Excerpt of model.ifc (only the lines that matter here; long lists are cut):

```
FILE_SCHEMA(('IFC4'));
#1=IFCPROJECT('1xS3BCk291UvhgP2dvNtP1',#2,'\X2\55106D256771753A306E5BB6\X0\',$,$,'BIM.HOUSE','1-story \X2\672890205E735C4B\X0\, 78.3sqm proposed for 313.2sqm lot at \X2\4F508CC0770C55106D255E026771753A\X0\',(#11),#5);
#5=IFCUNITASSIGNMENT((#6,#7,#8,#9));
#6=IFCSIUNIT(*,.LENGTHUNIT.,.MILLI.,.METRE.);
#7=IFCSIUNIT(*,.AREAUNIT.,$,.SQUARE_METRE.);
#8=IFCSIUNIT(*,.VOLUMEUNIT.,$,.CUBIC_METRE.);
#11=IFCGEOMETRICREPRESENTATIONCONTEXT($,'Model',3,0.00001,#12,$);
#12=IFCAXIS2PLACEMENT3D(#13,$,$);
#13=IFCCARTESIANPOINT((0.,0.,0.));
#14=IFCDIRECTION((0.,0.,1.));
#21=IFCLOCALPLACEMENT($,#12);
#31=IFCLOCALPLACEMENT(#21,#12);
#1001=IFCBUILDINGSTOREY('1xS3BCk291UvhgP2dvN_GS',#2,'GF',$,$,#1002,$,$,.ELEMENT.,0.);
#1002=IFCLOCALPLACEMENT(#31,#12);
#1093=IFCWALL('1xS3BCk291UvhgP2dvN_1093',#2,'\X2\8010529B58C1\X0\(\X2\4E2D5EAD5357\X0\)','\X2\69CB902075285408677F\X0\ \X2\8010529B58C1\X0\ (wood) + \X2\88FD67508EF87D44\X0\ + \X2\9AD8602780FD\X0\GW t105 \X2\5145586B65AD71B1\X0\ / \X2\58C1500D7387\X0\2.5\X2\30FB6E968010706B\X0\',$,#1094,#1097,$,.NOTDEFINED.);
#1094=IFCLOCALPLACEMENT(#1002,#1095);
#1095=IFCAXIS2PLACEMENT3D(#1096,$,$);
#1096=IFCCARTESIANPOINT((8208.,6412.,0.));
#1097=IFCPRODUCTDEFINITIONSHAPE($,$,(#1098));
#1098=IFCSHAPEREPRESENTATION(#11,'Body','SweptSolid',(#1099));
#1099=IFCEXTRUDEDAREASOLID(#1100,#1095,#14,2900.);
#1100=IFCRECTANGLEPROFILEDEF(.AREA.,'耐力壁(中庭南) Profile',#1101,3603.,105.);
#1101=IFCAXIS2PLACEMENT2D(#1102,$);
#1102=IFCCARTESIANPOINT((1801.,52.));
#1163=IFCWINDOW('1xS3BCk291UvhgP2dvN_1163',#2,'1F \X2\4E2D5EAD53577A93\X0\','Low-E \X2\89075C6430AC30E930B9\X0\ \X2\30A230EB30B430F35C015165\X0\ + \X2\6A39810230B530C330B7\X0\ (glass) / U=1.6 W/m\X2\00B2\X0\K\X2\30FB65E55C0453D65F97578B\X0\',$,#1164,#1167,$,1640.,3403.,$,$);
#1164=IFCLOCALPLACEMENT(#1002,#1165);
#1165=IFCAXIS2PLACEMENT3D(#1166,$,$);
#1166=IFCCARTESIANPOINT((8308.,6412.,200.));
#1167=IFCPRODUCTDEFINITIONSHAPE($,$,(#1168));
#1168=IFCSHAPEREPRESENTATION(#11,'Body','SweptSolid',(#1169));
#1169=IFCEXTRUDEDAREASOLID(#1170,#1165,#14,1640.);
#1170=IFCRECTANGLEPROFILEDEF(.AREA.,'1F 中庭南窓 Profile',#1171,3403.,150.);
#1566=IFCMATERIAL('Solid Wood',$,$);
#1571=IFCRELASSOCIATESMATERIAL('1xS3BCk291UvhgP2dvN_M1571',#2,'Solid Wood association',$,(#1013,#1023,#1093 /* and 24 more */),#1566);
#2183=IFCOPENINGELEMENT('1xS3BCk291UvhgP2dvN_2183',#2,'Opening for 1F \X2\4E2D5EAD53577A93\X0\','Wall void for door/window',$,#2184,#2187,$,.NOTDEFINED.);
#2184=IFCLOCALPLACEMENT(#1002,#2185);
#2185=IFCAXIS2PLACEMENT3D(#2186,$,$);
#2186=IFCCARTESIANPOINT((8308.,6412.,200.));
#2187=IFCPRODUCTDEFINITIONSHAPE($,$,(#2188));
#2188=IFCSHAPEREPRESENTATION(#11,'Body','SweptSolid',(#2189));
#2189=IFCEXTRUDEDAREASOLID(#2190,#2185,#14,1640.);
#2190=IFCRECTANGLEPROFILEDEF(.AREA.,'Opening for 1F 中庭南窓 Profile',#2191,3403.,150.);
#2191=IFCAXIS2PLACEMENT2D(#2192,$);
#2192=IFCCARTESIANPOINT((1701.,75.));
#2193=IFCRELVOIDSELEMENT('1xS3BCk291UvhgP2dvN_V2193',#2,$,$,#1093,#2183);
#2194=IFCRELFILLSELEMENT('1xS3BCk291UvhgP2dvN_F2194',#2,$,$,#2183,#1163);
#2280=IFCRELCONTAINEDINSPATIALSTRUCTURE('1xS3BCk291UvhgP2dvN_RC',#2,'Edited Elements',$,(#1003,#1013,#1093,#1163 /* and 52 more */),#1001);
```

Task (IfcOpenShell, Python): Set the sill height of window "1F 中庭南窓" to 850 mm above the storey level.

```python
import numpy as np
import ifcopenshell
import ifcopenshell.api.geometry
import ifcopenshell.geom
import ifcopenshell.util.element
import ifcopenshell.util.placement
import ifcopenshell.util.shape
import ifcopenshell.util.unit

model = ifcopenshell.open("model.ifc")
unit_scale = ifcopenshell.util.unit.calculate_unit_scale(model)

window = model.by_guid("1xS3BCk291UvhgP2dvN_1163")
opening = window.FillsVoids[0].RelatingOpeningElement
storey = ifcopenshell.util.element.get_container(window, ifc_class="IfcBuildingStorey")
level = ifcopenshell.util.placement.get_local_placement(storey.ObjectPlacement)[2, 3]

# The opening's origin need not be at the sill, so measure its lowest point.
shape = ifcopenshell.geom.create_shape(ifcopenshell.geom.settings(), opening)
bottom = ifcopenshell.util.shape.get_shape_bottom_elevation(shape, shape.geometry) / unit_scale
dz = level + 850.0 - bottom

shift = np.array([0.0, 0.0, dz])
# The window is not placed relative to its opening, so move both.
for product in (opening, window):
    matrix = ifcopenshell.util.placement.get_local_placement(product.ObjectPlacement)
    matrix[:3, 3] += shift
    ifcopenshell.api.geometry.edit_object_placement(model, product=product, matrix=matrix, is_si=False)

print(f"moved by {dz * unit_scale:+.3f} m")

model.write("model_updated.ifc")
```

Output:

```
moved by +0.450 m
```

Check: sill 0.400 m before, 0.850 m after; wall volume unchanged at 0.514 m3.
